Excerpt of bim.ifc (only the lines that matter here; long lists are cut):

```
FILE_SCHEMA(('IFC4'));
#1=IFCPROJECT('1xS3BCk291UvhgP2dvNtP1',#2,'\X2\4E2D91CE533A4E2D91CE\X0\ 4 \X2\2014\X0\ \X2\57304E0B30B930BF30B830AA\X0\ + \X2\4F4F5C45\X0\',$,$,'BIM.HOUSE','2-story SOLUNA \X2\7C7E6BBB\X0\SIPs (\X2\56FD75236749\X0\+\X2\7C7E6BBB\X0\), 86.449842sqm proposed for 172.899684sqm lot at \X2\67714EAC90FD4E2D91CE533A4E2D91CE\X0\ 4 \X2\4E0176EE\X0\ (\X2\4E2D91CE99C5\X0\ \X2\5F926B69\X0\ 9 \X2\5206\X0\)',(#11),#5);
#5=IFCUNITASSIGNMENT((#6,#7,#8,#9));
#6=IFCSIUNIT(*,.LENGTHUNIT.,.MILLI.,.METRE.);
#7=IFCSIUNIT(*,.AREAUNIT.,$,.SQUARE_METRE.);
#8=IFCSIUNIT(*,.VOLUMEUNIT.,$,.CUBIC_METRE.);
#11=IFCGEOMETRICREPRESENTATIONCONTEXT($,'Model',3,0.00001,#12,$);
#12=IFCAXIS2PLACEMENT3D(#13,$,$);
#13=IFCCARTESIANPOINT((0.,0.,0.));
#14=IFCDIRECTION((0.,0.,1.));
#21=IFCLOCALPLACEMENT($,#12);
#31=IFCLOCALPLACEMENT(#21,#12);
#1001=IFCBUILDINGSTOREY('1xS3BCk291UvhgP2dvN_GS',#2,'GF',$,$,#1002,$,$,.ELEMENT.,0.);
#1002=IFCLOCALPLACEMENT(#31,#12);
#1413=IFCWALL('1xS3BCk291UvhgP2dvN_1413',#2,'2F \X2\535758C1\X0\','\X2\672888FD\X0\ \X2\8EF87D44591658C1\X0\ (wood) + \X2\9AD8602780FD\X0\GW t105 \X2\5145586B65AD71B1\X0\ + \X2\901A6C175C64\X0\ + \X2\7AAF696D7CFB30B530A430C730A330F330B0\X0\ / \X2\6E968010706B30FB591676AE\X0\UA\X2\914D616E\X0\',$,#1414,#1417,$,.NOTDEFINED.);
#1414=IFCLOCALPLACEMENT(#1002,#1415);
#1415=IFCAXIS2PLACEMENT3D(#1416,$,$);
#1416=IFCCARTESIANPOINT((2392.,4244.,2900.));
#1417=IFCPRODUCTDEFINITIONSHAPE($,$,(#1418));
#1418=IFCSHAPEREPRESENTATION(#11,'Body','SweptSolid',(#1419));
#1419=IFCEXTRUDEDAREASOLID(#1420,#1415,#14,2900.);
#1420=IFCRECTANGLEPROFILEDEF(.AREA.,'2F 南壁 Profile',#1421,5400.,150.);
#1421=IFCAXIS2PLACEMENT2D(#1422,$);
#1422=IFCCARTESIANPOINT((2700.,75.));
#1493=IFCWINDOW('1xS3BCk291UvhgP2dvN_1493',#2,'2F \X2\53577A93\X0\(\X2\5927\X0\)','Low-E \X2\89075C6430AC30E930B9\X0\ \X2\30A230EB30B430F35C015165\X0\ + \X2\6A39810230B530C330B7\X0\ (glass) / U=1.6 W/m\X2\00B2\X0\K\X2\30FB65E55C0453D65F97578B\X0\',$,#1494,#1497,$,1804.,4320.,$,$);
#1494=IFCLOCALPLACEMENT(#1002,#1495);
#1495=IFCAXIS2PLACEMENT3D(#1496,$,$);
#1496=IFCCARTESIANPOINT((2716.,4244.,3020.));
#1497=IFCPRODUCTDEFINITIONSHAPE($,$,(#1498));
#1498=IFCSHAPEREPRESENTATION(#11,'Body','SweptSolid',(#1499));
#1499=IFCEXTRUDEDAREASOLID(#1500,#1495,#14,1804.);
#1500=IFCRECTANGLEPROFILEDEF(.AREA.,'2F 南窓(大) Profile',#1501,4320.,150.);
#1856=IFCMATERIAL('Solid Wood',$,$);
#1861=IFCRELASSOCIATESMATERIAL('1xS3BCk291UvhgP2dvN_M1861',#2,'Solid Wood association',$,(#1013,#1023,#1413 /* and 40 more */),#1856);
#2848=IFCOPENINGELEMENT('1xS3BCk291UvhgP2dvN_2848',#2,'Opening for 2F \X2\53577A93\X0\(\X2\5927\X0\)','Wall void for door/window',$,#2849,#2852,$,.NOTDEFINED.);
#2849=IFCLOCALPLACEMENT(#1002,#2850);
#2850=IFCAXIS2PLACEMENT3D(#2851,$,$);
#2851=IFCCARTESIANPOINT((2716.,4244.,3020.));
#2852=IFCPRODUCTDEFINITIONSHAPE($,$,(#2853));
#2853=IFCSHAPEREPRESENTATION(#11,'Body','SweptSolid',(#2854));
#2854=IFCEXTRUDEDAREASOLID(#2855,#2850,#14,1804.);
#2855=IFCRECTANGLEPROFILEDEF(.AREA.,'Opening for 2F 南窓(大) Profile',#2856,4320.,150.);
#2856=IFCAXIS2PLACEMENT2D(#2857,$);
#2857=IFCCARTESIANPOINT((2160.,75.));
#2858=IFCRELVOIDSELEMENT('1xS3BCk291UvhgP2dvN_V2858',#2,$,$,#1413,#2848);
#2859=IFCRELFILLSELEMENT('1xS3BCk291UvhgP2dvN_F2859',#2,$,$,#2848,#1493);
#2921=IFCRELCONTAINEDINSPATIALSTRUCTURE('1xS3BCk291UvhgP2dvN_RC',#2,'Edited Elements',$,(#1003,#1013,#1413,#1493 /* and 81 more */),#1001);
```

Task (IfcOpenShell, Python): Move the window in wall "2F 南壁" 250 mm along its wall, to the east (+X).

```python
import ifcopenshell
import ifcopenshell.api.geometry
import ifcopenshell.util.placement
import ifcopenshell.util.unit

model = ifcopenshell.open("bim.ifc")
unit_scale = ifcopenshell.util.unit.calculate_unit_scale(model)

window = model.by_guid("1xS3BCk291UvhgP2dvN_1493")
opening = window.FillsVoids[0].RelatingOpeningElement
wall = opening.VoidsElements[0].RelatingBuildingElement

wall_matrix = ifcopenshell.util.placement.get_local_placement(wall.ObjectPlacement)
shift = wall_matrix[:3, 0] * 0.25 / unit_scale
before = ifcopenshell.util.placement.get_local_placement(window.ObjectPlacement)[:3, 3].copy()

# The window is not placed relative to its opening, so move both.
for product in (opening, window):
    matrix = ifcopenshell.util.placement.get_local_placement(product.ObjectPlacement)
    matrix[:3, 3] += shift
    ifcopenshell.api.geometry.edit_object_placement(model, product=product, matrix=matrix, is_si=False)

after = ifcopenshell.util.placement.get_local_placement(window.ObjectPlacement)[:3, 3]
print("window moved by", (after - before).round(3) + 0.0)

model.write("bim_rev.ifc")
```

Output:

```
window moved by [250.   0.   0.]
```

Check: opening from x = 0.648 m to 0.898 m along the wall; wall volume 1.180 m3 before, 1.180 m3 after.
